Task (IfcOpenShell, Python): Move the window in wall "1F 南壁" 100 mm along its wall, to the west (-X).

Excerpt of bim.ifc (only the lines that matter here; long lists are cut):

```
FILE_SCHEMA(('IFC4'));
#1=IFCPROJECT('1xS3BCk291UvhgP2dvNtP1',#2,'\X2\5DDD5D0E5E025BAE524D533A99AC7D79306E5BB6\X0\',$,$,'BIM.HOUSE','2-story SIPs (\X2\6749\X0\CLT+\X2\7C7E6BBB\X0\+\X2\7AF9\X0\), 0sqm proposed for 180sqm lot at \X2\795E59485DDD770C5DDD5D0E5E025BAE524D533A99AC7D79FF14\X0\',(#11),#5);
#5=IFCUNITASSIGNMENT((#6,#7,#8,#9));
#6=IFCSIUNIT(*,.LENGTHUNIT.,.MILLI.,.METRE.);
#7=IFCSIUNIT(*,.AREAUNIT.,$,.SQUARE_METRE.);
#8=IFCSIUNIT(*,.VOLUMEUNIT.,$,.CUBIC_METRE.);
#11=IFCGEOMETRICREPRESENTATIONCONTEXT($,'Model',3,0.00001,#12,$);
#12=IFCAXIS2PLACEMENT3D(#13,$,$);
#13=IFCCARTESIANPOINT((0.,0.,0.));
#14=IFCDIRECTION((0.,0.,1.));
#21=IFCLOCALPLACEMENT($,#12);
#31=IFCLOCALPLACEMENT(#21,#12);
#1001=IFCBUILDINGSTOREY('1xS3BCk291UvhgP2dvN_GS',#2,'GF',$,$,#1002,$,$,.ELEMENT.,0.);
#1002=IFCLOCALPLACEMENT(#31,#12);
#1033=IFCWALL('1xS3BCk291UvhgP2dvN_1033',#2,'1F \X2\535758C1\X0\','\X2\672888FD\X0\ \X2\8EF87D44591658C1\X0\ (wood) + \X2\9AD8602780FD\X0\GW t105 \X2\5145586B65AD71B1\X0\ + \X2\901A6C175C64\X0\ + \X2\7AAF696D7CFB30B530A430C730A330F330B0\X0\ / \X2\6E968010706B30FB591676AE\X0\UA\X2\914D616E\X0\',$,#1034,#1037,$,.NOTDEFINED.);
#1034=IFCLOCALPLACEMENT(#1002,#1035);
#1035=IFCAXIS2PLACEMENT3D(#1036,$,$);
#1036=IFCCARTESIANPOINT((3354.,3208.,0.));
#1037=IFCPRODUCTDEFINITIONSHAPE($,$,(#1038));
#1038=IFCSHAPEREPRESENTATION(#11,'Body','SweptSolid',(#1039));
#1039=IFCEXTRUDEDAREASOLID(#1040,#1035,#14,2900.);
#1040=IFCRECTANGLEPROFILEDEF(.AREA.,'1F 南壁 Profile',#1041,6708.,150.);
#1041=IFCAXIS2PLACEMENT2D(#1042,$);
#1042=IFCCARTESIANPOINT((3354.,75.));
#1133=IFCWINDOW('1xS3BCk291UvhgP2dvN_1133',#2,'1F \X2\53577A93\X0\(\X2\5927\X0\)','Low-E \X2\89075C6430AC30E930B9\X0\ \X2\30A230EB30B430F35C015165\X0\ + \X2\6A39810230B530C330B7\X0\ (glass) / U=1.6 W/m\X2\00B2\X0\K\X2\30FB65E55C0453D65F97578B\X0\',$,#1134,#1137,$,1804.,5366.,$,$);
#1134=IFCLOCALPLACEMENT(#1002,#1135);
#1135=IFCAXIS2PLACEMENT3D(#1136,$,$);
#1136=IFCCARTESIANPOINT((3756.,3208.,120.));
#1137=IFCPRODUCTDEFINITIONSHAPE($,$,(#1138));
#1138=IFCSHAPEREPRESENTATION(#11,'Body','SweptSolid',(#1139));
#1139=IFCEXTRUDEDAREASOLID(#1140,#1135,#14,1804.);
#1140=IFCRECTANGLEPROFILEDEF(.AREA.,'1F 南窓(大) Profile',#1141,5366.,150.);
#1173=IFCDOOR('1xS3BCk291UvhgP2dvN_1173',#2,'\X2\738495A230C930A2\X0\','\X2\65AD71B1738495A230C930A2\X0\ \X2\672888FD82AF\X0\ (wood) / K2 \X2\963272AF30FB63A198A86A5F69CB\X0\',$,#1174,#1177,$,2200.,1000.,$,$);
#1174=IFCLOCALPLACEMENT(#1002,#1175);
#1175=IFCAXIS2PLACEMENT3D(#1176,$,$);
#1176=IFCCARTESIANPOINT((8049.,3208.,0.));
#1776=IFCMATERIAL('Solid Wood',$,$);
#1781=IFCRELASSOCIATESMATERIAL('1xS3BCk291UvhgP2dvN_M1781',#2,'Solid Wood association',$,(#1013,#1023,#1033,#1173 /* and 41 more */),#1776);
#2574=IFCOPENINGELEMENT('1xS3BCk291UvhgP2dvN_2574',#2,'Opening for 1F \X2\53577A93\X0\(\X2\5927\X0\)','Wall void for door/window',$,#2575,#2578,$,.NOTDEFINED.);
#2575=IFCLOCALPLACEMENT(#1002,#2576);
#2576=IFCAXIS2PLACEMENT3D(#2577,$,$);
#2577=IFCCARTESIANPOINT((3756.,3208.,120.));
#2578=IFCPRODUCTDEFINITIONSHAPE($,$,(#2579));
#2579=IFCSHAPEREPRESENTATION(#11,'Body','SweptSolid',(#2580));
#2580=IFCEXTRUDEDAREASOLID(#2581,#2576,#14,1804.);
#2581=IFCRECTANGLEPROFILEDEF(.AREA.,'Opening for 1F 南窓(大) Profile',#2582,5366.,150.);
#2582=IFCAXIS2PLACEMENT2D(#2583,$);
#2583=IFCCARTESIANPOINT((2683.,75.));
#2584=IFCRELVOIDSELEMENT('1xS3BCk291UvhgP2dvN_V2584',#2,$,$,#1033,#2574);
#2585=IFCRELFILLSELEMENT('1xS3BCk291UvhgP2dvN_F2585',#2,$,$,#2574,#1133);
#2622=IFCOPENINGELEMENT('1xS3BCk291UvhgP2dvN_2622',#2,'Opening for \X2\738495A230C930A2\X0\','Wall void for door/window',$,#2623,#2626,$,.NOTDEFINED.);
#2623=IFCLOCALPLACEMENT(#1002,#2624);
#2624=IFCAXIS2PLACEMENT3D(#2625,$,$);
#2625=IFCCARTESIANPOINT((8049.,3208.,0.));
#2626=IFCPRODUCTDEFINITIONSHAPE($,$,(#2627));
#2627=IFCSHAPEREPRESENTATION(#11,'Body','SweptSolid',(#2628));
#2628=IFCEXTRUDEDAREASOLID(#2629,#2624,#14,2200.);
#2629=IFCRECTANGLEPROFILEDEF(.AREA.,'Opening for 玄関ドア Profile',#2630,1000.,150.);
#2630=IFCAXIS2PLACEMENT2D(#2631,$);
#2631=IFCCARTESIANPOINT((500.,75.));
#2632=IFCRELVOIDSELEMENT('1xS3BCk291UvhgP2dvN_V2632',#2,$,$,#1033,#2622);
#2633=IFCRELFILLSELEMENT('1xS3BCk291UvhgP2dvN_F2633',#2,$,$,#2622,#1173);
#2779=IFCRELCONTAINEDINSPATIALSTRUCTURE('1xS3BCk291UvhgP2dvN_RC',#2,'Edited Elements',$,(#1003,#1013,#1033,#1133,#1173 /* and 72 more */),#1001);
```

```python
import ifcopenshell
import ifcopenshell.api.geometry
import ifcopenshell.util.placement
import ifcopenshell.util.unit

model = ifcopenshell.open("bim.ifc")
unit_scale = ifcopenshell.util.unit.calculate_unit_scale(model)

window = model.by_guid("1xS3BCk291UvhgP2dvN_1133")
opening = window.FillsVoids[0].RelatingOpeningElement
wall = opening.VoidsElements[0].RelatingBuildingElement

wall_matrix = ifcopenshell.util.placement.get_local_placement(wall.ObjectPlacement)
shift = wall_matrix[:3, 0] * -0.1 / unit_scale
before = ifcopenshell.util.placement.get_local_placement(window.ObjectPlacement)[:3, 3].copy()

# The window is not placed relative to its opening, so move both.
for product in (opening, window):
    matrix = ifcopenshell.util.placement.get_local_placement(product.ObjectPlacement)
    matrix[:3, 3] += shift
    ifcopenshell.api.geometry.edit_object_placement(model, product=product, matrix=matrix, is_si=False)

after = ifcopenshell.util.placement.get_local_placement(window.ObjectPlacement)[:3, 3]
print("window moved by", (after - before).round(3) + 0.0)

model.write("bim_updated.ifc")
```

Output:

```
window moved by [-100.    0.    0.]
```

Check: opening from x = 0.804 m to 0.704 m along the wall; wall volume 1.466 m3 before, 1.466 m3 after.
